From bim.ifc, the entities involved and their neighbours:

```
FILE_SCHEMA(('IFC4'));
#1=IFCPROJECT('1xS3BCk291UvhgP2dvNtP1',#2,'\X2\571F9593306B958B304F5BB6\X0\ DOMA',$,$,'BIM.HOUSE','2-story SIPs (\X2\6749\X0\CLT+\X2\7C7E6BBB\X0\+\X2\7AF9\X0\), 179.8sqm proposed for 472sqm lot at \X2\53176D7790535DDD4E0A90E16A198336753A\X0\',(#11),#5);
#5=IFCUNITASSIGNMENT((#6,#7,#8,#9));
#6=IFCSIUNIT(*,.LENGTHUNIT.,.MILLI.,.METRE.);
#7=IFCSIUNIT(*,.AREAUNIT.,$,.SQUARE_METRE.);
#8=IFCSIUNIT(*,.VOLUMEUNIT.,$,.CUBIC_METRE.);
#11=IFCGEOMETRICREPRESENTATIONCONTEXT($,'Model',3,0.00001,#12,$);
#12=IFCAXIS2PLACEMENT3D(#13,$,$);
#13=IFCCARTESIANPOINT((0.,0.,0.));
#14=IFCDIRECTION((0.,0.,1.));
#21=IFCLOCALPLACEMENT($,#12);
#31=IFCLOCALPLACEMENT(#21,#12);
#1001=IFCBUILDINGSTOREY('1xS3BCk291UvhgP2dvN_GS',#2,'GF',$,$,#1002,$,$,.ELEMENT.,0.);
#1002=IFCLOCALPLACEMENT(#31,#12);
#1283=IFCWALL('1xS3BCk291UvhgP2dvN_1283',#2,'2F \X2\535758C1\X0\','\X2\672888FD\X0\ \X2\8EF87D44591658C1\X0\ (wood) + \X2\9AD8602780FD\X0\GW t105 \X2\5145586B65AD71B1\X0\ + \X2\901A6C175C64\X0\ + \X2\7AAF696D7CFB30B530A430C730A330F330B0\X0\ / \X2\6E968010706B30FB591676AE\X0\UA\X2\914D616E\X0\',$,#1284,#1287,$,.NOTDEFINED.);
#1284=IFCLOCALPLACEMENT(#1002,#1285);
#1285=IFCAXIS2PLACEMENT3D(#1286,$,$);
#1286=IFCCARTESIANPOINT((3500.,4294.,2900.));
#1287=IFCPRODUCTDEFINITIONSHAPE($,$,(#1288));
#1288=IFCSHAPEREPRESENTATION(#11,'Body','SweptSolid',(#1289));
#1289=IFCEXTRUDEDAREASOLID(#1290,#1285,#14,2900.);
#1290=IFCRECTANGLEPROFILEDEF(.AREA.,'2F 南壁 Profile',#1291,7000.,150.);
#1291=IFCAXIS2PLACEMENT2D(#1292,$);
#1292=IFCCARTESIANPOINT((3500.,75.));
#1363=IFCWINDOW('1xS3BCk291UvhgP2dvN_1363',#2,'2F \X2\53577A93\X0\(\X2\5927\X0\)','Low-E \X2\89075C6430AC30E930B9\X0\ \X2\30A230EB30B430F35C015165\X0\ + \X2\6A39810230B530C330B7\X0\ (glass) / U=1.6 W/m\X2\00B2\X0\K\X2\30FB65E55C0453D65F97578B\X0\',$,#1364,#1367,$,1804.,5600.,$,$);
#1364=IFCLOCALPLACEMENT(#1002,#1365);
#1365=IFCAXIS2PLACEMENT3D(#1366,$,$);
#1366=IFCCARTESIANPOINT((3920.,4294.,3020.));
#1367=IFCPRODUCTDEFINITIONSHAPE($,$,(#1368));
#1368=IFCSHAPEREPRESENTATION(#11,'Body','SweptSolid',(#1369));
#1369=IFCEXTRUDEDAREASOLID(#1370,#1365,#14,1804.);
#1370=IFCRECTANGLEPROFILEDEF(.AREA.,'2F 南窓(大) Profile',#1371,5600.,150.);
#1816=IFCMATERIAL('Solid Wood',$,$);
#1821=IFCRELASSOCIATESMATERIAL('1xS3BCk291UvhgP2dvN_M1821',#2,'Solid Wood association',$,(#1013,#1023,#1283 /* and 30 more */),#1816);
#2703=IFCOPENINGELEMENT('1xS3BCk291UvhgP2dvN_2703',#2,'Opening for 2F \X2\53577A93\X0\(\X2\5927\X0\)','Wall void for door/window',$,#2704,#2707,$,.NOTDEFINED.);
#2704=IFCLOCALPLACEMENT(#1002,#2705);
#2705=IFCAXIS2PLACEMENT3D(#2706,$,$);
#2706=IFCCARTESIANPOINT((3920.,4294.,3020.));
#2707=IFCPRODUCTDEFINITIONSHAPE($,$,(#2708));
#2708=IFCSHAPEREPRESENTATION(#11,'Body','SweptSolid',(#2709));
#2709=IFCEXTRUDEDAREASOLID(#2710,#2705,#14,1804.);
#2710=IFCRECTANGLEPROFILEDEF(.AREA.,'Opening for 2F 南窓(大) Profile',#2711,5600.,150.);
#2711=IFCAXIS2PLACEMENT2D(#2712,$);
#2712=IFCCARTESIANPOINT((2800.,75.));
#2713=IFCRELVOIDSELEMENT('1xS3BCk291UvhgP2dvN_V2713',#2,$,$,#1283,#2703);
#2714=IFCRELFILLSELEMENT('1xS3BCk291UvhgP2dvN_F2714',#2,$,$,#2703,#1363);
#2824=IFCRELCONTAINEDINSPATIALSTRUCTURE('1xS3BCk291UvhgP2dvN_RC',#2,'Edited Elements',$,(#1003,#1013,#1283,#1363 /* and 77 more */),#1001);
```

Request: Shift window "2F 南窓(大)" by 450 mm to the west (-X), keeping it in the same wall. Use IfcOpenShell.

```python
import ifcopenshell
import ifcopenshell.api.geometry
import ifcopenshell.util.placement
import ifcopenshell.util.unit

model = ifcopenshell.open("bim.ifc")
unit_scale = ifcopenshell.util.unit.calculate_unit_scale(model)

window = model.by_id(1363)
opening = window.FillsVoids[0].RelatingOpeningElement
wall = opening.VoidsElements[0].RelatingBuildingElement

wall_matrix = ifcopenshell.util.placement.get_local_placement(wall.ObjectPlacement)
shift = wall_matrix[:3, 0] * -0.45 / unit_scale
before = ifcopenshell.util.placement.get_local_placement(window.ObjectPlacement)[:3, 3].copy()

# The window is not placed relative to its opening, so move both.
for product in (opening, window):
    matrix = ifcopenshell.util.placement.get_local_placement(product.ObjectPlacement)
    matrix[:3, 3] += shift
    ifcopenshell.api.geometry.edit_object_placement(model, product=product, matrix=matrix, is_si=False)

after = ifcopenshell.util.placement.get_local_placement(window.ObjectPlacement)[:3, 3]
print("window moved by", (after - before).round(3) + 0.0)

model.write("bim-out.ifc")
```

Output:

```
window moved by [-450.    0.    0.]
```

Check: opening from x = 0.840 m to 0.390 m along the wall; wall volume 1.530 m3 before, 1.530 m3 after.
